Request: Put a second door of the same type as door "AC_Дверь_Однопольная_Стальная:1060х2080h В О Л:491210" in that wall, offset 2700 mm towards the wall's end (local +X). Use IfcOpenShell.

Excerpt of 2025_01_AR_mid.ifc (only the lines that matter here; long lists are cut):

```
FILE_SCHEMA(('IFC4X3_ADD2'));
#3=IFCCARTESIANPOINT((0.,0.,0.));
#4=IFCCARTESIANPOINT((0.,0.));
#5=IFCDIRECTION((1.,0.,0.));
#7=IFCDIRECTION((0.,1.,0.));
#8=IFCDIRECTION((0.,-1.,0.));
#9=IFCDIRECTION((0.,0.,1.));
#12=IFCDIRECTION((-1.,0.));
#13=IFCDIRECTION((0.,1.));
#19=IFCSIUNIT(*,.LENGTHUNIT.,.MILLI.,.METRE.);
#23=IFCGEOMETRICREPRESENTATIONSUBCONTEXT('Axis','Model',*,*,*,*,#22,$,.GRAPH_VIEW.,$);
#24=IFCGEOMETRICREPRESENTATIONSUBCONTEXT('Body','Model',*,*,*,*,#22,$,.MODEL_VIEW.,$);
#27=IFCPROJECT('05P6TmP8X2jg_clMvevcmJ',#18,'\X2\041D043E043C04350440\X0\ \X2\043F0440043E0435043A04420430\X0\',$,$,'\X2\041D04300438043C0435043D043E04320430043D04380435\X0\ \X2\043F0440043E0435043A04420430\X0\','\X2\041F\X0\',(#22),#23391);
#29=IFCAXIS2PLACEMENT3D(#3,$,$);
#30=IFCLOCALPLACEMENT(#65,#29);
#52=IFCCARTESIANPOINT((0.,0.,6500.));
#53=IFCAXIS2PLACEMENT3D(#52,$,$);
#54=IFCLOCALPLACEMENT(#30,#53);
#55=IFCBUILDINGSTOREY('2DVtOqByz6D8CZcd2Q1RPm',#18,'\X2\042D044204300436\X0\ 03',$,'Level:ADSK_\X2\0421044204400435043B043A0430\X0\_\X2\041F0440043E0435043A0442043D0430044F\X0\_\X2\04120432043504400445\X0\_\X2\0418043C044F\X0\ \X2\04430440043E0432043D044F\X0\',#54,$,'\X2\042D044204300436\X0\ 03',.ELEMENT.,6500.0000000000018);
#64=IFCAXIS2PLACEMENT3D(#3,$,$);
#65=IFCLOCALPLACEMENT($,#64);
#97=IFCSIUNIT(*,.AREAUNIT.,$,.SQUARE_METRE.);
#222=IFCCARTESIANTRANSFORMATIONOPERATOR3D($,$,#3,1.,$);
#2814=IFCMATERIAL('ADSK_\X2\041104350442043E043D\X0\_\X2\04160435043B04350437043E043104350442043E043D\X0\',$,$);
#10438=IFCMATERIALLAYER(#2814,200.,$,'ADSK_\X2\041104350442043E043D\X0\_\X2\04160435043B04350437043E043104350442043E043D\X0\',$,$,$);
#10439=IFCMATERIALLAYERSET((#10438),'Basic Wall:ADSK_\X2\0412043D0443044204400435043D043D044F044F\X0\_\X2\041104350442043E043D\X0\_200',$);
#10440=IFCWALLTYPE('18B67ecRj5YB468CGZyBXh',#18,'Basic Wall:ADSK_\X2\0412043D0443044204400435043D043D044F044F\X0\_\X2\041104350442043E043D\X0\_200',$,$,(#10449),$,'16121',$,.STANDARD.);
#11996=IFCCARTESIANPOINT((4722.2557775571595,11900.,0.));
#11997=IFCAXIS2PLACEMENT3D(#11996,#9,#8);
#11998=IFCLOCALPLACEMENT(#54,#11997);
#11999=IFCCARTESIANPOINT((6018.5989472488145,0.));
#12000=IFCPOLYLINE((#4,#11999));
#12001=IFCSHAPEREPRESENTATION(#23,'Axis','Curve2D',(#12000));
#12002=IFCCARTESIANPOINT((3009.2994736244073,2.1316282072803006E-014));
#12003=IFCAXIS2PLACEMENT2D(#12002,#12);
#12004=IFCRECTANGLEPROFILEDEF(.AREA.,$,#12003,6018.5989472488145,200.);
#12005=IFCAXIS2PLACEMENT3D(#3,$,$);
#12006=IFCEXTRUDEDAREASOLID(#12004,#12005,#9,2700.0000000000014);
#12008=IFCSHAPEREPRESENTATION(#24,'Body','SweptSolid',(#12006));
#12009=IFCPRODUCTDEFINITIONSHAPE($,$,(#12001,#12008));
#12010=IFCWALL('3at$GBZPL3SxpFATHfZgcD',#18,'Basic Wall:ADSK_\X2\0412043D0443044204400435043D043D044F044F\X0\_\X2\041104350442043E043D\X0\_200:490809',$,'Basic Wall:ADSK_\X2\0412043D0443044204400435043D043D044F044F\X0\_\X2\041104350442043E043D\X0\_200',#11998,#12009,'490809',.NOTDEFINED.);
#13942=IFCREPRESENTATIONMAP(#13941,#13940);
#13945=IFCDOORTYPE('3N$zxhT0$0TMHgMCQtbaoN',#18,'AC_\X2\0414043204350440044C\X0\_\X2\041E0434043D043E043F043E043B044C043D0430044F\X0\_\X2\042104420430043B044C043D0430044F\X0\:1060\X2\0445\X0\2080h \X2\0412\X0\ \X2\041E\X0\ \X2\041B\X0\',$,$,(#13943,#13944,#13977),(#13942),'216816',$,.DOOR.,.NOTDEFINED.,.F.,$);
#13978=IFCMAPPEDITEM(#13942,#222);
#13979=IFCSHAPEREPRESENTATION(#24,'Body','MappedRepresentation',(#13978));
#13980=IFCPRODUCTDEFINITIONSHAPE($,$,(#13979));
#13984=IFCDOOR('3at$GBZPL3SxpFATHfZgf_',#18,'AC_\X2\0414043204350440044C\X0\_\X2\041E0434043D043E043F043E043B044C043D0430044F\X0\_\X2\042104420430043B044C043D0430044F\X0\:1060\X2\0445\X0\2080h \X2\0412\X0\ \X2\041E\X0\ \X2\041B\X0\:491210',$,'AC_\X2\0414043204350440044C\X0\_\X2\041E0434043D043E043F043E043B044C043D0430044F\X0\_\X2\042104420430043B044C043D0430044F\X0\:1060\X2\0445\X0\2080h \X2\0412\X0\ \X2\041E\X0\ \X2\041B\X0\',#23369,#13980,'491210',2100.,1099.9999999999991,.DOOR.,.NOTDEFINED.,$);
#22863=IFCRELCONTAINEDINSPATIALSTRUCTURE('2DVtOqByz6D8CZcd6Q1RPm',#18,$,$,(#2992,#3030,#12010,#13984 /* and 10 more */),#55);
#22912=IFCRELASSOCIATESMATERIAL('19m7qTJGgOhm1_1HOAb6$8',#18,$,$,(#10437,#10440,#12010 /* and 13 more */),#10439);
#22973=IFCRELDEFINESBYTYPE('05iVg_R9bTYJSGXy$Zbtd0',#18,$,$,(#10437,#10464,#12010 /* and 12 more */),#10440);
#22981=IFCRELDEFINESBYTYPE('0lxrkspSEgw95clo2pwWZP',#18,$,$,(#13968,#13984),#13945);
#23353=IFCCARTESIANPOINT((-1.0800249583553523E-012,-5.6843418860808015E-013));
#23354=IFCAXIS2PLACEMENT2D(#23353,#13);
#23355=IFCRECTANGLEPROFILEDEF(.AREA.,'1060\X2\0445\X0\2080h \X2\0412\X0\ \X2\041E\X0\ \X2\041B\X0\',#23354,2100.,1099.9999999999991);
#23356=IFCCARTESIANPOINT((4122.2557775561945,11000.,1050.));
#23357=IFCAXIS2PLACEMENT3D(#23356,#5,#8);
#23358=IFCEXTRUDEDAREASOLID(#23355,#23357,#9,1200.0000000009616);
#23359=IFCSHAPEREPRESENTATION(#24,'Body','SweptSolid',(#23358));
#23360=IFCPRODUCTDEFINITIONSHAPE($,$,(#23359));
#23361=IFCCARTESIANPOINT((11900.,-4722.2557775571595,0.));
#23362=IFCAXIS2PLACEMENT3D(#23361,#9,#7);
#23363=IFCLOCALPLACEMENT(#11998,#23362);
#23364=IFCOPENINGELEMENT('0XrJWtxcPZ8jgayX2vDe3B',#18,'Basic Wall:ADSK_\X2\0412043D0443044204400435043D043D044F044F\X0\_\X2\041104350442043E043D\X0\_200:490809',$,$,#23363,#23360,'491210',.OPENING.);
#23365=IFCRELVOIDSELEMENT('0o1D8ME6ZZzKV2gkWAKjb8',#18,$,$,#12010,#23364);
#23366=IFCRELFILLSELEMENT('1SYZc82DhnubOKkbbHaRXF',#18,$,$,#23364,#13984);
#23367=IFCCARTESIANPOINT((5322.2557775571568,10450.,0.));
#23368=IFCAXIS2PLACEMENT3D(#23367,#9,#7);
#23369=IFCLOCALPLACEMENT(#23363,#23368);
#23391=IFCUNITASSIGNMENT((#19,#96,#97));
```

```python
import ifcopenshell
import ifcopenshell.api.feature
import ifcopenshell.api.geometry
import ifcopenshell.api.root
import ifcopenshell.geom
import ifcopenshell.util.element
import ifcopenshell.util.placement
import ifcopenshell.util.shape

model = ifcopenshell.open("2025_01_AR_mid.ifc")
settings = ifcopenshell.geom.settings()


def volume(element):
    """Net volume in cubic metres, openings subtracted."""
    shape = ifcopenshell.geom.create_shape(settings, element)
    return ifcopenshell.util.shape.get_volume(shape.geometry)


def reuse_history(source, copy):
    """copy_class also copies each property set's owner history, people and application; keep the originals."""
    for rel in copy.IsDefinedBy:
        if rel.is_a("IfcRelDefinesByProperties") and (history := rel.RelatingPropertyDefinition.OwnerHistory):
            rel.RelatingPropertyDefinition.OwnerHistory = source.OwnerHistory
            ifcopenshell.util.element.remove_deep2(model, history)


door = model.by_guid("3at$GBZPL3SxpFATHfZgf_")
opening = door.FillsVoids[0].RelatingOpeningElement
wall = opening.VoidsElements[0].RelatingBuildingElement
before = volume(wall)
shift = ifcopenshell.util.placement.get_local_placement(wall.ObjectPlacement)[:3, 0] * 2700.0

# copy_class copies the void relationship, type, container and properties, but no geometry.
new_opening = ifcopenshell.api.root.copy_class(model, product=opening)
new_opening.Representation = ifcopenshell.util.element.copy_deep(
    model, opening.Representation, exclude=["IfcGeometricRepresentationContext", "IfcRepresentationMap"]
)
new_opening.Name = "Basic Wall:ADSK_Внутренняя_Бетон_200"
new_opening.Tag = None
new_door = ifcopenshell.api.root.copy_class(model, product=door)
new_door.Representation = ifcopenshell.util.element.copy_deep(
    model, door.Representation, exclude=["IfcGeometricRepresentationContext", "IfcRepresentationMap"]
)
new_door.Name = "AC_Дверь_Однопольная_Стальная:1060х2080h В О Л"
new_door.Tag = None
reuse_history(door, new_door)
ifcopenshell.api.feature.add_filling(model, opening=new_opening, element=new_door)

for old, new in ((opening, new_opening), (door, new_door)):
    matrix = ifcopenshell.util.placement.get_local_placement(old.ObjectPlacement)
    matrix[:3, 3] += shift
    ifcopenshell.api.geometry.edit_object_placement(model, product=new, matrix=matrix, is_si=False)

after = volume(wall)

print(f"wall volume {before:.3f} -> {after:.3f} m3")

model.write("2025_01_AR_mid_v2.ifc")
```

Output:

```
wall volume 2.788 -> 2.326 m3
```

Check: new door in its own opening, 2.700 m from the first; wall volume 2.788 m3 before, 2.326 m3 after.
